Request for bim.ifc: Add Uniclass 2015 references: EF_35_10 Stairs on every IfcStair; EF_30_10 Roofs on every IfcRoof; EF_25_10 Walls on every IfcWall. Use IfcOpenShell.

First a look at what the model holds.

```python
import ifcopenshell

model = ifcopenshell.open("bim.ifc")
print(model.schema)
print("classifications:", [c.Name for c in model.by_type("IfcClassification")])
for ifc_class in ("IfcDoor", "IfcRoof", "IfcStair", "IfcWall", "IfcWindow"):
    print(ifc_class, len(model.by_type(ifc_class)))
```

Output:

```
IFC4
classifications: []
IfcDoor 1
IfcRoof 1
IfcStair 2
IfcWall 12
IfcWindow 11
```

```python
import ifcopenshell
import ifcopenshell.api.classification

model = ifcopenshell.open("bim.ifc")

system = ifcopenshell.api.classification.add_classification(model, classification="Uniclass 2015")

codes = {
    "IfcStair": ("EF_35_10", "Stairs"),
    "IfcRoof": ("EF_30_10", "Roofs"),
    "IfcWall": ("EF_25_10", "Walls"),
}
for ifc_class, (code, name) in codes.items():
    products = model.by_type(ifc_class)
    ifcopenshell.api.classification.add_reference(
        model, products=products, classification=system, identification=code, name=name
    )
    print(code, len(products))

model.write("bim-out.ifc")
```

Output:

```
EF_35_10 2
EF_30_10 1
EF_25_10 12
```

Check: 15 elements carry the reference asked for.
